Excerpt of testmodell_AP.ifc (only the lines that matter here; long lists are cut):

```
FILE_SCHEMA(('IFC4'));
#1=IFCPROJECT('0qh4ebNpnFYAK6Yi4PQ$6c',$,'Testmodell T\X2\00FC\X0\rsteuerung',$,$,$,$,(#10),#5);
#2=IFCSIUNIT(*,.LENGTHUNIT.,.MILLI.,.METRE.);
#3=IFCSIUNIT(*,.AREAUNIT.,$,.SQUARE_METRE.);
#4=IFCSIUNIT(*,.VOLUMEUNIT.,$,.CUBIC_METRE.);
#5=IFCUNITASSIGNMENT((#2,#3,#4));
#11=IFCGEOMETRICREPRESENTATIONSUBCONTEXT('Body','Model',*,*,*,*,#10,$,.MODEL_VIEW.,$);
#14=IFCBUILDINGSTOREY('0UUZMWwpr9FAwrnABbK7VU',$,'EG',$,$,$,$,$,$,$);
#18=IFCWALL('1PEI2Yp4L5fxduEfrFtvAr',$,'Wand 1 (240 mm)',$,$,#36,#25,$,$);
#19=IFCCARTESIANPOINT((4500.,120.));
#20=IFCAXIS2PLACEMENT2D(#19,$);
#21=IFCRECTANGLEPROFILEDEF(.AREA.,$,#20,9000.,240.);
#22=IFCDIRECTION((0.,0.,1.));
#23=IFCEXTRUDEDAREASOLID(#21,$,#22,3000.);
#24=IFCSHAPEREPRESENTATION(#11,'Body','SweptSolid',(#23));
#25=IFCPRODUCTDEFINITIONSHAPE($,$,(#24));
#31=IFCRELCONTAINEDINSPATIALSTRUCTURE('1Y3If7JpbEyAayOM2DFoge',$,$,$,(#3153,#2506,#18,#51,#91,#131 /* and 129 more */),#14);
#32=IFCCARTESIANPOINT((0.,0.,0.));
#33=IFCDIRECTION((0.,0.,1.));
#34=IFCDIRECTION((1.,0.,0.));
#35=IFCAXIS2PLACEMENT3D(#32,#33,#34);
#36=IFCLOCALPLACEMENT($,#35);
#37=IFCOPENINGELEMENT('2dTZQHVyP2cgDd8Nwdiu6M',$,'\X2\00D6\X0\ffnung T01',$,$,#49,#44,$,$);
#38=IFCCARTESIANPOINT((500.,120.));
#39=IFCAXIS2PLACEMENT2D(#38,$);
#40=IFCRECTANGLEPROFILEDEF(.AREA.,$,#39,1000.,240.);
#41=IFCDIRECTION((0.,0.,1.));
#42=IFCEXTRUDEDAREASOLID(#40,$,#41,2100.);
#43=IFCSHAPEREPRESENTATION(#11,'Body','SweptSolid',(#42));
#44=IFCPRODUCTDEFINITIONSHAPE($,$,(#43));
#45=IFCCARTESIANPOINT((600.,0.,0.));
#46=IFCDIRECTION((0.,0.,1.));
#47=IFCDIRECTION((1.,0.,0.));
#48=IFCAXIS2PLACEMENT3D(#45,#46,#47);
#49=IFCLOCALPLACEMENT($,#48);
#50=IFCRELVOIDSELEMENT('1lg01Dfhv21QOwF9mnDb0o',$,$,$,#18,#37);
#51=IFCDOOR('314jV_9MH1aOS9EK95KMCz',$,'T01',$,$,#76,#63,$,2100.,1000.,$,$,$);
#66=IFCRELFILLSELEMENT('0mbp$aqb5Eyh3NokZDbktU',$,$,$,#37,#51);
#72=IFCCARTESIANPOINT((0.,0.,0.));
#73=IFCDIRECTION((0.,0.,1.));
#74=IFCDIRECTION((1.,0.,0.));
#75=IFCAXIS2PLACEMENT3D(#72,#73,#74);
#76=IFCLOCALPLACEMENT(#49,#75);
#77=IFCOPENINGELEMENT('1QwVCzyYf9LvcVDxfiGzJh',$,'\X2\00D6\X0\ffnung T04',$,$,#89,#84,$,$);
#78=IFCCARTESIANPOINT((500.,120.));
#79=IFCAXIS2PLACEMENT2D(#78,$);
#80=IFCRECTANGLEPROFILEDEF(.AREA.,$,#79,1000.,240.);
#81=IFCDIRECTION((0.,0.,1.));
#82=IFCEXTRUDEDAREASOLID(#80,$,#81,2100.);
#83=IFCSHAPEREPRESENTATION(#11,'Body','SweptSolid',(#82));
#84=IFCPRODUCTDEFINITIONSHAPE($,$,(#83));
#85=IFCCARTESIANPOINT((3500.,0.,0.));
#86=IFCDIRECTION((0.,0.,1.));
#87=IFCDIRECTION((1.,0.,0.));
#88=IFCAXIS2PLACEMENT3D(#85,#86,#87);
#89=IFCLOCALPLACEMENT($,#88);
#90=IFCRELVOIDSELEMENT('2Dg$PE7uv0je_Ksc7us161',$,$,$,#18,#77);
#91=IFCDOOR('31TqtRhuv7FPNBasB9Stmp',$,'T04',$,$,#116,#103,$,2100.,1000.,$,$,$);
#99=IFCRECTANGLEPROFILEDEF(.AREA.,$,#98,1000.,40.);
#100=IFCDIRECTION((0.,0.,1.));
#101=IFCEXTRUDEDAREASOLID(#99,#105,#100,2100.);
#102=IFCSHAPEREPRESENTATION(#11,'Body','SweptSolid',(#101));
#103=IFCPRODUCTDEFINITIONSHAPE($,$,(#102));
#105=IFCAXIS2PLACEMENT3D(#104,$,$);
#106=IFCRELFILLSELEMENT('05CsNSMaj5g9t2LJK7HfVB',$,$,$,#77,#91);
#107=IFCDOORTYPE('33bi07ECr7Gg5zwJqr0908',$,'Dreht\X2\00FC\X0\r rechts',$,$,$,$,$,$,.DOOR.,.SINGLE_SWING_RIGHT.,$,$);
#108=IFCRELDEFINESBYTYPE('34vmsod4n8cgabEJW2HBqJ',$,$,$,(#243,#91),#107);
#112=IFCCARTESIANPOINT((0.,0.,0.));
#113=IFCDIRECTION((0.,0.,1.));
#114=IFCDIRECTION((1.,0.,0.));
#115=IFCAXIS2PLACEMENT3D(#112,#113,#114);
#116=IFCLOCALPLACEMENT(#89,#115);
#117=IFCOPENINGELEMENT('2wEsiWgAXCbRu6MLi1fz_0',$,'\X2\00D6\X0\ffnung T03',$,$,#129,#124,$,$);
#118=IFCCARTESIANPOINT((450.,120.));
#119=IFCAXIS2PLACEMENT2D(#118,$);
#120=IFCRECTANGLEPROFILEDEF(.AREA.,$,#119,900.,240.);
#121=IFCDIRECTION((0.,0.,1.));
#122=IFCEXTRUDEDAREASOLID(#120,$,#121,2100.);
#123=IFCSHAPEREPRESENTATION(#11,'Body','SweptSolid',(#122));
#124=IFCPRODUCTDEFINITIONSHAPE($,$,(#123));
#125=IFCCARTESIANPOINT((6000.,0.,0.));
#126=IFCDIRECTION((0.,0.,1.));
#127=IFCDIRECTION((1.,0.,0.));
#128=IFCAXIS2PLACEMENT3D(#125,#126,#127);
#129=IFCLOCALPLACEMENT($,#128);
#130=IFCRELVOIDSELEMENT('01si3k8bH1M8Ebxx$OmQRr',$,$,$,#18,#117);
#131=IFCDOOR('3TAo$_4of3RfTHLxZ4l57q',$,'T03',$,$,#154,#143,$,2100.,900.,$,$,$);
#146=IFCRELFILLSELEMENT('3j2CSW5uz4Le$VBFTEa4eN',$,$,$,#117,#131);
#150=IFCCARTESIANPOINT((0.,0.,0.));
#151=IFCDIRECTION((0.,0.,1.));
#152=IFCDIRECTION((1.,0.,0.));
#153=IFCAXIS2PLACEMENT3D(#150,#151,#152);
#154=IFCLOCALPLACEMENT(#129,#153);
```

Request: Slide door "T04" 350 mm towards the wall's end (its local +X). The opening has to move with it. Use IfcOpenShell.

```python
import ifcopenshell
import ifcopenshell.api.geometry
import ifcopenshell.util.placement
import ifcopenshell.util.unit

model = ifcopenshell.open("testmodell_AP.ifc")
unit_scale = ifcopenshell.util.unit.calculate_unit_scale(model)

door = model.by_id(91)
opening = door.FillsVoids[0].RelatingOpeningElement
wall = opening.VoidsElements[0].RelatingBuildingElement

wall_matrix = ifcopenshell.util.placement.get_local_placement(wall.ObjectPlacement)
shift = wall_matrix[:3, 0] * 0.35 / unit_scale
before = ifcopenshell.util.placement.get_local_placement(door.ObjectPlacement)[:3, 3].copy()

# The door is placed relative to its opening, so it follows when the opening moves.
matrix = ifcopenshell.util.placement.get_local_placement(opening.ObjectPlacement)
matrix[:3, 3] += shift
ifcopenshell.api.geometry.edit_object_placement(
    model, product=opening, matrix=matrix, is_si=False, should_transform_children=True
)

after = ifcopenshell.util.placement.get_local_placement(door.ObjectPlacement)[:3, 3]
print("door moved by", (after - before).round(3) + 0.0)

model.write("testmodell_AP_edited.ifc")
```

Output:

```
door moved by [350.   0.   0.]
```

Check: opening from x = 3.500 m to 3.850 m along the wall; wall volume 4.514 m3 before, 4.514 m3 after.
